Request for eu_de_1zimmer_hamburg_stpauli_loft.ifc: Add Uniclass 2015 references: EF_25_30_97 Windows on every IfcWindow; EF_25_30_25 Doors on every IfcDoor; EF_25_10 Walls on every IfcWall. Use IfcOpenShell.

First a look at what the model holds.

```python
import ifcopenshell

model = ifcopenshell.open("eu_de_1zimmer_hamburg_stpauli_loft.ifc")
print(model.schema)
print("classifications:", [c.Name for c in model.by_type("IfcClassification")])
for ifc_class in ("IfcDoor", "IfcRoof", "IfcStair", "IfcWall", "IfcWindow"):
    print(ifc_class, len(model.by_type(ifc_class)))
```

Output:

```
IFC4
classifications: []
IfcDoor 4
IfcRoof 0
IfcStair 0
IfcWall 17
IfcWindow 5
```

```python
import ifcopenshell
import ifcopenshell.api.classification

model = ifcopenshell.open("eu_de_1zimmer_hamburg_stpauli_loft.ifc")

system = ifcopenshell.api.classification.add_classification(model, classification="Uniclass 2015")

codes = {
    "IfcWindow": ("EF_25_30_97", "Windows"),
    "IfcDoor": ("EF_25_30_25", "Doors"),
    "IfcWall": ("EF_25_10", "Walls"),
}
for ifc_class, (code, name) in codes.items():
    products = model.by_type(ifc_class)
    ifcopenshell.api.classification.add_reference(
        model, products=products, classification=system, identification=code, name=name
    )
    print(code, len(products))

model.write("eu_de_1zimmer_hamburg_stpauli_loft_rev.ifc")
```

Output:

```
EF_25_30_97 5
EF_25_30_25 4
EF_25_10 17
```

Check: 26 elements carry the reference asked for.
